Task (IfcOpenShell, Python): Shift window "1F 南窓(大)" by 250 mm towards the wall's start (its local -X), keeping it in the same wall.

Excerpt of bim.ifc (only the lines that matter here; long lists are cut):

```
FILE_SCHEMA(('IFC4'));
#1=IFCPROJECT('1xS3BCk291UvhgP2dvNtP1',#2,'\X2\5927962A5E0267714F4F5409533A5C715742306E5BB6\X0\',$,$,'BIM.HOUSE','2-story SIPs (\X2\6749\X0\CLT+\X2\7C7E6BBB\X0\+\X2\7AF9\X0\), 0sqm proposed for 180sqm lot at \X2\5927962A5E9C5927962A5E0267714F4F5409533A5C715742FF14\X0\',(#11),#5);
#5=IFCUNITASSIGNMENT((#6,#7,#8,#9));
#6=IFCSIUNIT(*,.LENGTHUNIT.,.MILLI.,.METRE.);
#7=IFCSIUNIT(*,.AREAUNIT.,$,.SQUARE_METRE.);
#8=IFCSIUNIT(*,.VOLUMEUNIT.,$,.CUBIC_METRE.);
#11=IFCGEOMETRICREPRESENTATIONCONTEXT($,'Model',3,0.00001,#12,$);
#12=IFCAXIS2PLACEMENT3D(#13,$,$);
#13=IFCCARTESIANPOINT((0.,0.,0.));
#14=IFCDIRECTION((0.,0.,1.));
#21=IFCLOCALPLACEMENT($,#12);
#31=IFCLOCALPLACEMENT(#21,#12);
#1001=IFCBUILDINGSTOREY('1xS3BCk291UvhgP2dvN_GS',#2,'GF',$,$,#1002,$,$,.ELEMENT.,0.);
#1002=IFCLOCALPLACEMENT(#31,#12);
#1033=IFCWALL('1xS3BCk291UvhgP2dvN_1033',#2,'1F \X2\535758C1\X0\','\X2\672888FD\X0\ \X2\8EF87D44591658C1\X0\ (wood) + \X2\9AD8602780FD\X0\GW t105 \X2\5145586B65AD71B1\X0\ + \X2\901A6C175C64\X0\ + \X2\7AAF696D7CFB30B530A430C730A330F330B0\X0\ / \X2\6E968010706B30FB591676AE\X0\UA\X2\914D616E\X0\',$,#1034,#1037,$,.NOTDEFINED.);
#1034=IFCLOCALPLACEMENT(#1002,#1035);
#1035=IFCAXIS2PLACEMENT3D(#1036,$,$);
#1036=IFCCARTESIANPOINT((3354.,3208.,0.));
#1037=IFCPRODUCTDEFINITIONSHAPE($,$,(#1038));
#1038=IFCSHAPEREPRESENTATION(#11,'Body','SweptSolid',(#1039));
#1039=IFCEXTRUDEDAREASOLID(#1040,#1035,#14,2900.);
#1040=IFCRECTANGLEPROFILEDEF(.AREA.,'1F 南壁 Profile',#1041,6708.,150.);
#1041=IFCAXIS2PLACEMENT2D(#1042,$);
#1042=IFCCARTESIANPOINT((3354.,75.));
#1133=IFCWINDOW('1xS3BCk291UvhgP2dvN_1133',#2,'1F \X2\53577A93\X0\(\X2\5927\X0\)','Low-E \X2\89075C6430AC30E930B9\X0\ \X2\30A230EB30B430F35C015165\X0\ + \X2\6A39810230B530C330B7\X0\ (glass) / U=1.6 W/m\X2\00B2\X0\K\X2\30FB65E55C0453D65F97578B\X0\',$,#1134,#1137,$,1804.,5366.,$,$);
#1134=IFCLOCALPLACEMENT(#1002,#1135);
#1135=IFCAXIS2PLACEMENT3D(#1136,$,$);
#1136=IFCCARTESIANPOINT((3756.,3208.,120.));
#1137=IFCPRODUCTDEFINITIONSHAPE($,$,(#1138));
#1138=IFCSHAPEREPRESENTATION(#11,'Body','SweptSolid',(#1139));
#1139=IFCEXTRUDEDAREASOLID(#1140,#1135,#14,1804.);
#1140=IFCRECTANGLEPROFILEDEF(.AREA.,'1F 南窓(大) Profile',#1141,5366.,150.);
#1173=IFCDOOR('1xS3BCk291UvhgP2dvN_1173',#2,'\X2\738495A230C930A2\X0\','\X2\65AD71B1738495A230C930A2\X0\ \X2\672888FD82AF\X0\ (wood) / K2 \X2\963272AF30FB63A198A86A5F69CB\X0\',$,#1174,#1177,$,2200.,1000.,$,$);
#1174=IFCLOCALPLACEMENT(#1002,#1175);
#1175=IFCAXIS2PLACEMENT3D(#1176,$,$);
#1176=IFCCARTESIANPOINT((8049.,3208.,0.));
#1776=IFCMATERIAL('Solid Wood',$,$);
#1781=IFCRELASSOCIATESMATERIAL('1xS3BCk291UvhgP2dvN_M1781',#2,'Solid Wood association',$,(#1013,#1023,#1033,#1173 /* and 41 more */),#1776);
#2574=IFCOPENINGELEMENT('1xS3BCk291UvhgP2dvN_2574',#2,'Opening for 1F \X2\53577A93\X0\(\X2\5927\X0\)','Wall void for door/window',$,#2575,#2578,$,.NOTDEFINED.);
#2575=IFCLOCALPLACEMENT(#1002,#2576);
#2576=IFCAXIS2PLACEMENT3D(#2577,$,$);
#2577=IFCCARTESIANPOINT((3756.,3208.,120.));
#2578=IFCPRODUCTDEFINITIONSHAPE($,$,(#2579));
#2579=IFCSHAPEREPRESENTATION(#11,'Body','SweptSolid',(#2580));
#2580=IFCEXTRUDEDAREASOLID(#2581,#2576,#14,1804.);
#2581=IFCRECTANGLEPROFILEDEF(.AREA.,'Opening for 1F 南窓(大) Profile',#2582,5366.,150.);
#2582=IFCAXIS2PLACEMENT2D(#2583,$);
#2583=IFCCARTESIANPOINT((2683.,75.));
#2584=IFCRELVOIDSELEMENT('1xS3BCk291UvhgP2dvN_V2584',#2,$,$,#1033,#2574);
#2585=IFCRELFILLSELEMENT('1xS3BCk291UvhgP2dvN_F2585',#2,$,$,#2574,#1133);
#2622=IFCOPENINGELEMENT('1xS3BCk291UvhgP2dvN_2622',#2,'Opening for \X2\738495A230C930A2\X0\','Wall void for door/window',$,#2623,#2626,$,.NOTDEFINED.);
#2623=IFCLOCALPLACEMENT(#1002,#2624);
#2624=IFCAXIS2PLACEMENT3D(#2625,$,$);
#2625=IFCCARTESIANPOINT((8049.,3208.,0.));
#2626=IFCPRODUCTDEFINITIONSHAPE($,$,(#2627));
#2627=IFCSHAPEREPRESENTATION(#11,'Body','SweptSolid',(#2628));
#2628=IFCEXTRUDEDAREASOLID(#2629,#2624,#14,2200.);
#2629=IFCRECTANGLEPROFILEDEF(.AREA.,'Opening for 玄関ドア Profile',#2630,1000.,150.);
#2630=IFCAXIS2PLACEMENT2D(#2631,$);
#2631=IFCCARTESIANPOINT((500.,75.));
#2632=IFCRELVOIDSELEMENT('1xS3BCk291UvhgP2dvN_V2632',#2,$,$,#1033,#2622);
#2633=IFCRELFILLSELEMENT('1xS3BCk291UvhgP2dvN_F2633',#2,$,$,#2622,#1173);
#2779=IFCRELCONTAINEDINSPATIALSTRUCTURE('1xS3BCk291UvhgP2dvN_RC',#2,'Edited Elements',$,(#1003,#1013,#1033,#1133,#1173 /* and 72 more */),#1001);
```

```python
import ifcopenshell
import ifcopenshell.api.geometry
import ifcopenshell.util.placement

model = ifcopenshell.open("bim.ifc")

window = model.by_id(1133)
opening = window.FillsVoids[0].RelatingOpeningElement
wall = opening.VoidsElements[0].RelatingBuildingElement

wall_matrix = ifcopenshell.util.placement.get_local_placement(wall.ObjectPlacement)
shift = wall_matrix[:3, 0] * -250.0
before = ifcopenshell.util.placement.get_local_placement(window.ObjectPlacement)[:3, 3].copy()

# The window is not placed relative to its opening, so move both.
for product in (opening, window):
    matrix = ifcopenshell.util.placement.get_local_placement(product.ObjectPlacement)
    matrix[:3, 3] += shift
    ifcopenshell.api.geometry.edit_object_placement(model, product=product, matrix=matrix, is_si=False)

after = ifcopenshell.util.placement.get_local_placement(window.ObjectPlacement)[:3, 3]
print("window moved by", (after - before).round(3) + 0.0)

model.write("bim-out.ifc")
```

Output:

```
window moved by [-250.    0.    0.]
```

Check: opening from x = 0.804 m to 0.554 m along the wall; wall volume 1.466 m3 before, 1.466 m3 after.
